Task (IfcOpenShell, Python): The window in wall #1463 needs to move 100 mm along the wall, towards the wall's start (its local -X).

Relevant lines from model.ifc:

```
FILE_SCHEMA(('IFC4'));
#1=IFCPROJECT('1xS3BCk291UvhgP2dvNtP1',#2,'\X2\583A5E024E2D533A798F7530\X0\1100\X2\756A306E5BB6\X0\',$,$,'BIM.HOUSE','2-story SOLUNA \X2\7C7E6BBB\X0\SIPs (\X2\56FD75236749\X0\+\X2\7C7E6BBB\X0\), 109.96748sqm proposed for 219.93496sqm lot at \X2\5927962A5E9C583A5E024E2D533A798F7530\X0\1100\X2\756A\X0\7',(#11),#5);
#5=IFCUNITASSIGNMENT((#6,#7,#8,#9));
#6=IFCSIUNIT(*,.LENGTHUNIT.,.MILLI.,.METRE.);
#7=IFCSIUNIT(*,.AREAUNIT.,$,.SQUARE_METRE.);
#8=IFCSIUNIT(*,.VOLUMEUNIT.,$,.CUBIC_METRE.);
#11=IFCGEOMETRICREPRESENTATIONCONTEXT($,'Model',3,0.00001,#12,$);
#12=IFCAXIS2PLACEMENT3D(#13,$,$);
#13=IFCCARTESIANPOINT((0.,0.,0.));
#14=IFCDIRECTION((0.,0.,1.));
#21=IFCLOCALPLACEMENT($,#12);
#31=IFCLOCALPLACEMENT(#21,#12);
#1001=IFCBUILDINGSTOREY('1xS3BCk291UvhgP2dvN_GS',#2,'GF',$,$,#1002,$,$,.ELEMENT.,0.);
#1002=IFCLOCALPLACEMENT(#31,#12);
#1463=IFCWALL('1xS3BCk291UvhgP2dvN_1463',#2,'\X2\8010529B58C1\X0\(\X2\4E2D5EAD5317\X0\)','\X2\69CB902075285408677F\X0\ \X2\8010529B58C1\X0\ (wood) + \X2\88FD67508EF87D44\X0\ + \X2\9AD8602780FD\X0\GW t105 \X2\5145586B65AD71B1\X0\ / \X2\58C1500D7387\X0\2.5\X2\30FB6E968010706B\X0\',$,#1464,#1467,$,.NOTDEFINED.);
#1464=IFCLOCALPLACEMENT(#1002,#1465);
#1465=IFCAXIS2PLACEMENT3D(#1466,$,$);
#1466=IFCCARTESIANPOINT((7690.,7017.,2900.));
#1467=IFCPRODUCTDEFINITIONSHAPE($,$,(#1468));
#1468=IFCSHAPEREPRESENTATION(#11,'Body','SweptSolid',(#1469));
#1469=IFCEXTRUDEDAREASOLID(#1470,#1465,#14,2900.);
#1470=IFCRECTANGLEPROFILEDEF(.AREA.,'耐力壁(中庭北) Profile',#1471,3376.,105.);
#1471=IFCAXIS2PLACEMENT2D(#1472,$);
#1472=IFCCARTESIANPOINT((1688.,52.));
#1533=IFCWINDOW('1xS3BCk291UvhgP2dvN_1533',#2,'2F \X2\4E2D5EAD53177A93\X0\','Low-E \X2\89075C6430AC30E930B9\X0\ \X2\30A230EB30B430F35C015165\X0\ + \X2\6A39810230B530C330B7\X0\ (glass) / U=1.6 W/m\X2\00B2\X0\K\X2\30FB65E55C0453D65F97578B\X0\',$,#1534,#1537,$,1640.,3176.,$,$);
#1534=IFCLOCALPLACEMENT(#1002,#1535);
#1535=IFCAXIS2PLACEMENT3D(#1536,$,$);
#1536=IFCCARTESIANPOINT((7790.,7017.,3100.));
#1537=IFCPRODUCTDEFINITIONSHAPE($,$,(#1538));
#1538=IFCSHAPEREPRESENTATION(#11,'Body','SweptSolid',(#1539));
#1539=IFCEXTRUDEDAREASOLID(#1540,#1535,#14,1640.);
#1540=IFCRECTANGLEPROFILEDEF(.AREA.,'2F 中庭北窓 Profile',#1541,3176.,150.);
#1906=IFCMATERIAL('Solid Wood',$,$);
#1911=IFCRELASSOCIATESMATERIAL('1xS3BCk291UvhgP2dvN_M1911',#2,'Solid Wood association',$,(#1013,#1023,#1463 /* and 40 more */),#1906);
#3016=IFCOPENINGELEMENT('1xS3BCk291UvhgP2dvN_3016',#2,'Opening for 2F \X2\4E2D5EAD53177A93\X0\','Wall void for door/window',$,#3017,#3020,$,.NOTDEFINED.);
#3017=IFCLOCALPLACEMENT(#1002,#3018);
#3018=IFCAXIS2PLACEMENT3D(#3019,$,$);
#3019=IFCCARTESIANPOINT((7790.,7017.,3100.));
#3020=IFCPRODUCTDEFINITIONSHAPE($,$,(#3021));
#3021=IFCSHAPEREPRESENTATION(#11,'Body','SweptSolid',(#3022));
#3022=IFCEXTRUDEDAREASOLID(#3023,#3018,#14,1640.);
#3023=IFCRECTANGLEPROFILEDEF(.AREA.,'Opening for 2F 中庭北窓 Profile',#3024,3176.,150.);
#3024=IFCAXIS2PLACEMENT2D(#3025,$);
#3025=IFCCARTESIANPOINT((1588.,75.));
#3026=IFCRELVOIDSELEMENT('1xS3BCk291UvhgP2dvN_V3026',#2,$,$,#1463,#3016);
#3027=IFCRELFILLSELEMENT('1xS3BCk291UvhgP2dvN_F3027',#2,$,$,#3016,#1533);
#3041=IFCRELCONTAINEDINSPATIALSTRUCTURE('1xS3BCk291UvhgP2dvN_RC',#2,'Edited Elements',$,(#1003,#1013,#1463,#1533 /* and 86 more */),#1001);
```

```python
import ifcopenshell
import ifcopenshell.api.geometry
import ifcopenshell.util.placement

model = ifcopenshell.open("model.ifc")

window = model.by_guid("1xS3BCk291UvhgP2dvN_1533")
opening = window.FillsVoids[0].RelatingOpeningElement
wall = opening.VoidsElements[0].RelatingBuildingElement

wall_matrix = ifcopenshell.util.placement.get_local_placement(wall.ObjectPlacement)
shift = wall_matrix[:3, 0] * -100.0
before = ifcopenshell.util.placement.get_local_placement(window.ObjectPlacement)[:3, 3].copy()

# The window is not placed relative to its opening, so move both.
for product in (opening, window):
    matrix = ifcopenshell.util.placement.get_local_placement(product.ObjectPlacement)
    matrix[:3, 3] += shift
    ifcopenshell.api.geometry.edit_object_placement(model, product=product, matrix=matrix, is_si=False)

after = ifcopenshell.util.placement.get_local_placement(window.ObjectPlacement)[:3, 3]
print("window moved by", (after - before).round(3) + 0.0)

model.write("model_v2.ifc")
```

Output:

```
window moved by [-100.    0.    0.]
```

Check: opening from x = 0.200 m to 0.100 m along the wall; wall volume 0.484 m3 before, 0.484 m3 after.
